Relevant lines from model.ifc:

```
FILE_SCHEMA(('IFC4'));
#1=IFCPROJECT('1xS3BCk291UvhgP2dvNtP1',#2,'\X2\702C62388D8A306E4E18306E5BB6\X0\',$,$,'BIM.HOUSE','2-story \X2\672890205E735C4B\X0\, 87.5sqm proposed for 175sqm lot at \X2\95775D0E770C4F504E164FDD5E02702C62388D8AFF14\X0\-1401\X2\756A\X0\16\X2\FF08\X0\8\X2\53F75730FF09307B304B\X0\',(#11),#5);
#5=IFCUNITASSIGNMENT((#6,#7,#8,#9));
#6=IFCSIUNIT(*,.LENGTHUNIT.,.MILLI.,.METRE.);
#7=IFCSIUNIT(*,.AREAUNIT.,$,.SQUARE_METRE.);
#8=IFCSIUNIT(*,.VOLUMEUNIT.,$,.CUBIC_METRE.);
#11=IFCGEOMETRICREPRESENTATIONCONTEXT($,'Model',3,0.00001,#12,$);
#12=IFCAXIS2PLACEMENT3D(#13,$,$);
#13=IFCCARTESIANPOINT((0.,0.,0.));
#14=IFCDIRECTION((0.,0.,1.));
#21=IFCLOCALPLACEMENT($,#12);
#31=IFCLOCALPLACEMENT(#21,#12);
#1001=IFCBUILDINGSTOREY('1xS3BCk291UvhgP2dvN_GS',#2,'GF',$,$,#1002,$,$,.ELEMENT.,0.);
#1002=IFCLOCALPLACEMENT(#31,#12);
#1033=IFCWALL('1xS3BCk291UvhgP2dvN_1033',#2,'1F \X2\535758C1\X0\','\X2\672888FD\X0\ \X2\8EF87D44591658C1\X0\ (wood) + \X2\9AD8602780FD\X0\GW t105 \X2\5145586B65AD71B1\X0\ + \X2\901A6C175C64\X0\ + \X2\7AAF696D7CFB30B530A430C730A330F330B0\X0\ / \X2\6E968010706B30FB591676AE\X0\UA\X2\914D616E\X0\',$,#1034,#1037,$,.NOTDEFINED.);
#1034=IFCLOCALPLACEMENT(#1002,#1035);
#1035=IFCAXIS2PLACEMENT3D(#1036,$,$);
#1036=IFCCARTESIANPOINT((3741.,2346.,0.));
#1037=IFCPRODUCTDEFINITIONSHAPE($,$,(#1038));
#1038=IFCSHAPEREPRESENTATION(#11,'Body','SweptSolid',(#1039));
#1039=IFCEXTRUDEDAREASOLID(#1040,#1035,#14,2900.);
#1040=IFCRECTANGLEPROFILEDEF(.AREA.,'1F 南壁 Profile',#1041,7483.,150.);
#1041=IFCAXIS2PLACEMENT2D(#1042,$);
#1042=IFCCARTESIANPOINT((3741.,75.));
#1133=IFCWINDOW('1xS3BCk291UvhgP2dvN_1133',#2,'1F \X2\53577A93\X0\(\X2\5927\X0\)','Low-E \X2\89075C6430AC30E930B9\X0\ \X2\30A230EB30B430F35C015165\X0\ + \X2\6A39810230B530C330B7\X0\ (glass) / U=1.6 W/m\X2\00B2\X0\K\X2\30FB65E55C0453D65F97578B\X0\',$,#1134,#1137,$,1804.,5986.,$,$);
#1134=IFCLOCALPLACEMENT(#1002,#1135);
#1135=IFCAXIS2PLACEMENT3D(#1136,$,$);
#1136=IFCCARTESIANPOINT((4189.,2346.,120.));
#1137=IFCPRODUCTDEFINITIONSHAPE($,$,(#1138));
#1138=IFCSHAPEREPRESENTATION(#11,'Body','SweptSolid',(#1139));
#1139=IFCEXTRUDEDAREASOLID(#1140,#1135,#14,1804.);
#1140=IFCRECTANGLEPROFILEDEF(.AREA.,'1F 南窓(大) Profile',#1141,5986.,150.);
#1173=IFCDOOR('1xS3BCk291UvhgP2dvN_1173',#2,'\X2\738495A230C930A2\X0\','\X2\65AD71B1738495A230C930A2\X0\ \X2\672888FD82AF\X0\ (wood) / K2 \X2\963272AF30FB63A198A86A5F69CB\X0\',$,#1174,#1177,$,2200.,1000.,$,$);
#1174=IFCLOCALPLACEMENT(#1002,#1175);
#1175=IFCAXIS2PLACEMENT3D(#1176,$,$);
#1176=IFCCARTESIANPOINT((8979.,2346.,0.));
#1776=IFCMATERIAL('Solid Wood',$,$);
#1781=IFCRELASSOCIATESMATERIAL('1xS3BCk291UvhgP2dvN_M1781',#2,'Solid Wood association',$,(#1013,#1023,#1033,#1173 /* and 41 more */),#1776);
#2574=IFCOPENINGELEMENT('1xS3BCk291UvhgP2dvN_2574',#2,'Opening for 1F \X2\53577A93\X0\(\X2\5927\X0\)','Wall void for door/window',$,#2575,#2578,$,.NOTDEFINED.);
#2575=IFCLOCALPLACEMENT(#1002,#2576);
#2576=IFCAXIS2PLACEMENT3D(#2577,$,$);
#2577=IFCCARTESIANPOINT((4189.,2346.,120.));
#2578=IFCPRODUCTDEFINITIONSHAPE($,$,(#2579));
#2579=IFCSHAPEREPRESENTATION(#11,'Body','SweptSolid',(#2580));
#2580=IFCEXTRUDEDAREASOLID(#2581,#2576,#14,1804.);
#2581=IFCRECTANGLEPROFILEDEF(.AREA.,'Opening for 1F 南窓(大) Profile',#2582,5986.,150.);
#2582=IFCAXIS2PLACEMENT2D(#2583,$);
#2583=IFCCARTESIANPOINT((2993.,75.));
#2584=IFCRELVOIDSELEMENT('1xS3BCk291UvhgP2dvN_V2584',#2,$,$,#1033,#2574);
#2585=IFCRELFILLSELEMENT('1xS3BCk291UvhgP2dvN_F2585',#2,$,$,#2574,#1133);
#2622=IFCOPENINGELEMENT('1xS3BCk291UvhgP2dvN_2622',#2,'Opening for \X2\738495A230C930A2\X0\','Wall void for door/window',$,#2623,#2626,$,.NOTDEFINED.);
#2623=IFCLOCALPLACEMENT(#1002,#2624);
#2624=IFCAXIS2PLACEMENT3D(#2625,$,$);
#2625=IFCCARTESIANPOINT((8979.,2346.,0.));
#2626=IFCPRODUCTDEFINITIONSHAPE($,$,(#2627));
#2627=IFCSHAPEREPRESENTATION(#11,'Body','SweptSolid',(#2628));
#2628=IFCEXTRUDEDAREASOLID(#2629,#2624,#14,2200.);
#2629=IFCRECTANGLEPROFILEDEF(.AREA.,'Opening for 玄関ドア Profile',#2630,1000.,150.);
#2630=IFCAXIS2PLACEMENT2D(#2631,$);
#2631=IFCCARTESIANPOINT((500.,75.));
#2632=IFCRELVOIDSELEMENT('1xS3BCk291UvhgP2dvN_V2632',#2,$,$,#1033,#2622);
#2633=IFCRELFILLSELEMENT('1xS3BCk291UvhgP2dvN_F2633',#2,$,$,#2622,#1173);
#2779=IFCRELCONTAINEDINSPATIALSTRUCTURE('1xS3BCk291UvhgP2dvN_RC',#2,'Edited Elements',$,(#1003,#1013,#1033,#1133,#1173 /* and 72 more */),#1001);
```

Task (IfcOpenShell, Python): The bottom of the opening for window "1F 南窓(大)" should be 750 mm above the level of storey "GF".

```python
import numpy as np
import ifcopenshell
import ifcopenshell.api.geometry
import ifcopenshell.geom
import ifcopenshell.util.element
import ifcopenshell.util.placement
import ifcopenshell.util.shape
import ifcopenshell.util.unit

model = ifcopenshell.open("model.ifc")
unit_scale = ifcopenshell.util.unit.calculate_unit_scale(model)

window = model.by_guid("1xS3BCk291UvhgP2dvN_1133")
opening = window.FillsVoids[0].RelatingOpeningElement
storey = ifcopenshell.util.element.get_container(window, ifc_class="IfcBuildingStorey")
level = ifcopenshell.util.placement.get_local_placement(storey.ObjectPlacement)[2, 3]

# The opening's origin need not be at the sill, so measure its lowest point.
shape = ifcopenshell.geom.create_shape(ifcopenshell.geom.settings(), opening)
bottom = ifcopenshell.util.shape.get_shape_bottom_elevation(shape, shape.geometry) / unit_scale
dz = level + 750.0 - bottom

shift = np.array([0.0, 0.0, dz])
# The window is not placed relative to its opening, so move both.
for product in (opening, window):
    matrix = ifcopenshell.util.placement.get_local_placement(product.ObjectPlacement)
    matrix[:3, 3] += shift
    ifcopenshell.api.geometry.edit_object_placement(model, product=product, matrix=matrix, is_si=False)

print(f"moved by {dz * unit_scale:+.3f} m")

model.write("model_updated.ifc")
```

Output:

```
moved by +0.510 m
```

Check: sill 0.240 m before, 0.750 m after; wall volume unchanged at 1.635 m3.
